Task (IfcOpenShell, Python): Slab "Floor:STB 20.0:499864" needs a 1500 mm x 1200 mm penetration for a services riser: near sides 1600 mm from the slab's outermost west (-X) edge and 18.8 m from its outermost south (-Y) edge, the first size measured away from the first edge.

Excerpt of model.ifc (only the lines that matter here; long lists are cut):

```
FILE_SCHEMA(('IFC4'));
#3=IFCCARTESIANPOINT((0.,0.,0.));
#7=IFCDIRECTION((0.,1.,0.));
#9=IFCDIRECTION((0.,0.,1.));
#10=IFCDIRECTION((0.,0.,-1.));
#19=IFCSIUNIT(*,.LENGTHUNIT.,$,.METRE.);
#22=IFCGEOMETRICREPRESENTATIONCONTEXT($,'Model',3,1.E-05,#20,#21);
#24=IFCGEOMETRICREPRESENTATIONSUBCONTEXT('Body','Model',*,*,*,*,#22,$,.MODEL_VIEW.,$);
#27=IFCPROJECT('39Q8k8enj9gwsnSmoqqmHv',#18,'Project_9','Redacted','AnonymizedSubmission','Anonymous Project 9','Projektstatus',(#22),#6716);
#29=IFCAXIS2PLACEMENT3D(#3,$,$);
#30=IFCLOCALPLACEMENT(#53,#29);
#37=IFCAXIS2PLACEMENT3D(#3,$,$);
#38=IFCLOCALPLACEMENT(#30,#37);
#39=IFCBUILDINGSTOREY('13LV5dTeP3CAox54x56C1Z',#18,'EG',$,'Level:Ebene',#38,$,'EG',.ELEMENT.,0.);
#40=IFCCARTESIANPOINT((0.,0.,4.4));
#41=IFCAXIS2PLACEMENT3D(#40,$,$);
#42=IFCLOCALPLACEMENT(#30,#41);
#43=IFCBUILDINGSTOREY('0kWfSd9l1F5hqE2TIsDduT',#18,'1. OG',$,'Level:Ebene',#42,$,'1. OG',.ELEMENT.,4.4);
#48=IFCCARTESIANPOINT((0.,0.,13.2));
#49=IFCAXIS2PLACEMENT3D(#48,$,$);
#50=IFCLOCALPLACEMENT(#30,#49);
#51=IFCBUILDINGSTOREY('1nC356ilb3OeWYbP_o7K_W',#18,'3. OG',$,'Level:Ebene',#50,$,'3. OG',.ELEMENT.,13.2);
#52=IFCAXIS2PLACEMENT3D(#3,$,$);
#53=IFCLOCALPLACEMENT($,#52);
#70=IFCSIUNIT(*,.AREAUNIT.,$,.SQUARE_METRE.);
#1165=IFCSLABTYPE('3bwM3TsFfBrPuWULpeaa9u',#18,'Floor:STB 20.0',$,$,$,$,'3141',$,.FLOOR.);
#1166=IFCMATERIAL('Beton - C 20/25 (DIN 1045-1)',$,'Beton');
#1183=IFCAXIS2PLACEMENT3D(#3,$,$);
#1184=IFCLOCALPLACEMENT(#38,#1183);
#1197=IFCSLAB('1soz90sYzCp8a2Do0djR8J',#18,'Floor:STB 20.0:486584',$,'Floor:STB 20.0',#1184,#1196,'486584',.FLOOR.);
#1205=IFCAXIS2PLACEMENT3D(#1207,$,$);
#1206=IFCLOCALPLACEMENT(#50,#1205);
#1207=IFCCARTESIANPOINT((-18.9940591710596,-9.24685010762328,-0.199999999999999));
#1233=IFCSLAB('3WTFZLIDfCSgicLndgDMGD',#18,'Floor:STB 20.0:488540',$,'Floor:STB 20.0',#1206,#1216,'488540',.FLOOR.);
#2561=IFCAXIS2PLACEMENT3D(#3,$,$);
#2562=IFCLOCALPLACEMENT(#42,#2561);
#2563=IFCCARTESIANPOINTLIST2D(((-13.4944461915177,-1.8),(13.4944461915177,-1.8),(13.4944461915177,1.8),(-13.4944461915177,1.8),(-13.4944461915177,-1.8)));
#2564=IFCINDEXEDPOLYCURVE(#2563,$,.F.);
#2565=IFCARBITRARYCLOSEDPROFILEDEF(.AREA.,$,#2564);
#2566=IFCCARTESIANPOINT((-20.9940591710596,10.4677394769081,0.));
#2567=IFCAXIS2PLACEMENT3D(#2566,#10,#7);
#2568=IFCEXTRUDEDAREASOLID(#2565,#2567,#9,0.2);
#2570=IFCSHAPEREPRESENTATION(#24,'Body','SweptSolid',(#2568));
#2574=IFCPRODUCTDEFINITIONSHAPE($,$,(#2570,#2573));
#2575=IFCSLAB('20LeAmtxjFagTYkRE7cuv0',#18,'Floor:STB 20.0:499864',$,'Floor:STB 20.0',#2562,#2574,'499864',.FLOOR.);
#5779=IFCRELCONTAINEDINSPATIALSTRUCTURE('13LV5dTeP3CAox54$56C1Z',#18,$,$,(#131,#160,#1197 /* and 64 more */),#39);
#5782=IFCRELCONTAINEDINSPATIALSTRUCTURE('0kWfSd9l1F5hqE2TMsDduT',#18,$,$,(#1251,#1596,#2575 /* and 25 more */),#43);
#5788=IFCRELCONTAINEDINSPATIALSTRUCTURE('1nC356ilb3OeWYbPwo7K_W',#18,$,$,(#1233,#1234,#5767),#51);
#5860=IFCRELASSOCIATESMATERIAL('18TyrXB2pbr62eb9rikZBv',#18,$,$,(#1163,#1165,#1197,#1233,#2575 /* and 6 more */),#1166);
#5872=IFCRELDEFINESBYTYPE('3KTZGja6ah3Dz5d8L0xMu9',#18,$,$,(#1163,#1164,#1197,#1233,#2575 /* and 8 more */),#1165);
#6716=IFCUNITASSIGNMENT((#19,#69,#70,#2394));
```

```python
import numpy as np
import ifcopenshell
import ifcopenshell.api.feature
import ifcopenshell.api.geometry
import ifcopenshell.api.root
import ifcopenshell.geom
import ifcopenshell.util.placement
import ifcopenshell.util.representation
import ifcopenshell.util.shape
import ifcopenshell.util.unit

model = ifcopenshell.open("model.ifc")
unit_scale = ifcopenshell.util.unit.calculate_unit_scale(model)
settings = ifcopenshell.geom.settings()


def volume(element):
    """Net volume in cubic metres, openings subtracted."""
    shape = ifcopenshell.geom.create_shape(settings, element)
    return ifcopenshell.util.shape.get_volume(shape.geometry)


slab = model.by_guid("20LeAmtxjFagTYkRE7cuv0")
before = volume(slab)

# Extent in the slab's own axes, in metres. The edges named are its -X and -Y sides.
slab_shape = ifcopenshell.geom.create_shape(settings, slab)
vertices = ifcopenshell.util.shape.get_vertices(slab_shape.geometry)
x_min, y_min, bottom = vertices.min(axis=0)
top = vertices[:, 2].max()

opening = ifcopenshell.api.root.create_entity(model, ifc_class="IfcOpeningElement", name="Services riser opening", predefined_type="OPENING")
context = ifcopenshell.util.representation.get_context(model, "Model", "Body", "MODEL_VIEW")
width, depth = 1.5, 1.2
outline = [(0.0, 0.0), (width, 0.0), (width, depth), (0.0, depth), (0.0, 0.0)]
# Overshoot both faces by 50 mm so the cut is clean.
shape = ifcopenshell.api.geometry.add_slab_representation(
    model, context=context, depth=top - bottom + 0.1, polyline=outline
)
ifcopenshell.api.geometry.assign_representation(model, product=opening, representation=shape)

matrix = ifcopenshell.util.placement.get_local_placement(slab.ObjectPlacement)
matrix[:, 3] = matrix @ np.append(np.array([x_min + 1.6, y_min + 18.8, bottom - 0.05]) / unit_scale, 1.0)
ifcopenshell.api.geometry.edit_object_placement(model, product=opening, matrix=matrix, is_si=False)
ifcopenshell.api.feature.add_feature(model, feature=opening, element=slab)

after = volume(slab)

print(f"slab volume {before:.3f} -> {after:.3f} m3")

model.write("model_v2.ifc")
```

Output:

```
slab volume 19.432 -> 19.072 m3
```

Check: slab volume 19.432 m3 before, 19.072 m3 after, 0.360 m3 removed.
